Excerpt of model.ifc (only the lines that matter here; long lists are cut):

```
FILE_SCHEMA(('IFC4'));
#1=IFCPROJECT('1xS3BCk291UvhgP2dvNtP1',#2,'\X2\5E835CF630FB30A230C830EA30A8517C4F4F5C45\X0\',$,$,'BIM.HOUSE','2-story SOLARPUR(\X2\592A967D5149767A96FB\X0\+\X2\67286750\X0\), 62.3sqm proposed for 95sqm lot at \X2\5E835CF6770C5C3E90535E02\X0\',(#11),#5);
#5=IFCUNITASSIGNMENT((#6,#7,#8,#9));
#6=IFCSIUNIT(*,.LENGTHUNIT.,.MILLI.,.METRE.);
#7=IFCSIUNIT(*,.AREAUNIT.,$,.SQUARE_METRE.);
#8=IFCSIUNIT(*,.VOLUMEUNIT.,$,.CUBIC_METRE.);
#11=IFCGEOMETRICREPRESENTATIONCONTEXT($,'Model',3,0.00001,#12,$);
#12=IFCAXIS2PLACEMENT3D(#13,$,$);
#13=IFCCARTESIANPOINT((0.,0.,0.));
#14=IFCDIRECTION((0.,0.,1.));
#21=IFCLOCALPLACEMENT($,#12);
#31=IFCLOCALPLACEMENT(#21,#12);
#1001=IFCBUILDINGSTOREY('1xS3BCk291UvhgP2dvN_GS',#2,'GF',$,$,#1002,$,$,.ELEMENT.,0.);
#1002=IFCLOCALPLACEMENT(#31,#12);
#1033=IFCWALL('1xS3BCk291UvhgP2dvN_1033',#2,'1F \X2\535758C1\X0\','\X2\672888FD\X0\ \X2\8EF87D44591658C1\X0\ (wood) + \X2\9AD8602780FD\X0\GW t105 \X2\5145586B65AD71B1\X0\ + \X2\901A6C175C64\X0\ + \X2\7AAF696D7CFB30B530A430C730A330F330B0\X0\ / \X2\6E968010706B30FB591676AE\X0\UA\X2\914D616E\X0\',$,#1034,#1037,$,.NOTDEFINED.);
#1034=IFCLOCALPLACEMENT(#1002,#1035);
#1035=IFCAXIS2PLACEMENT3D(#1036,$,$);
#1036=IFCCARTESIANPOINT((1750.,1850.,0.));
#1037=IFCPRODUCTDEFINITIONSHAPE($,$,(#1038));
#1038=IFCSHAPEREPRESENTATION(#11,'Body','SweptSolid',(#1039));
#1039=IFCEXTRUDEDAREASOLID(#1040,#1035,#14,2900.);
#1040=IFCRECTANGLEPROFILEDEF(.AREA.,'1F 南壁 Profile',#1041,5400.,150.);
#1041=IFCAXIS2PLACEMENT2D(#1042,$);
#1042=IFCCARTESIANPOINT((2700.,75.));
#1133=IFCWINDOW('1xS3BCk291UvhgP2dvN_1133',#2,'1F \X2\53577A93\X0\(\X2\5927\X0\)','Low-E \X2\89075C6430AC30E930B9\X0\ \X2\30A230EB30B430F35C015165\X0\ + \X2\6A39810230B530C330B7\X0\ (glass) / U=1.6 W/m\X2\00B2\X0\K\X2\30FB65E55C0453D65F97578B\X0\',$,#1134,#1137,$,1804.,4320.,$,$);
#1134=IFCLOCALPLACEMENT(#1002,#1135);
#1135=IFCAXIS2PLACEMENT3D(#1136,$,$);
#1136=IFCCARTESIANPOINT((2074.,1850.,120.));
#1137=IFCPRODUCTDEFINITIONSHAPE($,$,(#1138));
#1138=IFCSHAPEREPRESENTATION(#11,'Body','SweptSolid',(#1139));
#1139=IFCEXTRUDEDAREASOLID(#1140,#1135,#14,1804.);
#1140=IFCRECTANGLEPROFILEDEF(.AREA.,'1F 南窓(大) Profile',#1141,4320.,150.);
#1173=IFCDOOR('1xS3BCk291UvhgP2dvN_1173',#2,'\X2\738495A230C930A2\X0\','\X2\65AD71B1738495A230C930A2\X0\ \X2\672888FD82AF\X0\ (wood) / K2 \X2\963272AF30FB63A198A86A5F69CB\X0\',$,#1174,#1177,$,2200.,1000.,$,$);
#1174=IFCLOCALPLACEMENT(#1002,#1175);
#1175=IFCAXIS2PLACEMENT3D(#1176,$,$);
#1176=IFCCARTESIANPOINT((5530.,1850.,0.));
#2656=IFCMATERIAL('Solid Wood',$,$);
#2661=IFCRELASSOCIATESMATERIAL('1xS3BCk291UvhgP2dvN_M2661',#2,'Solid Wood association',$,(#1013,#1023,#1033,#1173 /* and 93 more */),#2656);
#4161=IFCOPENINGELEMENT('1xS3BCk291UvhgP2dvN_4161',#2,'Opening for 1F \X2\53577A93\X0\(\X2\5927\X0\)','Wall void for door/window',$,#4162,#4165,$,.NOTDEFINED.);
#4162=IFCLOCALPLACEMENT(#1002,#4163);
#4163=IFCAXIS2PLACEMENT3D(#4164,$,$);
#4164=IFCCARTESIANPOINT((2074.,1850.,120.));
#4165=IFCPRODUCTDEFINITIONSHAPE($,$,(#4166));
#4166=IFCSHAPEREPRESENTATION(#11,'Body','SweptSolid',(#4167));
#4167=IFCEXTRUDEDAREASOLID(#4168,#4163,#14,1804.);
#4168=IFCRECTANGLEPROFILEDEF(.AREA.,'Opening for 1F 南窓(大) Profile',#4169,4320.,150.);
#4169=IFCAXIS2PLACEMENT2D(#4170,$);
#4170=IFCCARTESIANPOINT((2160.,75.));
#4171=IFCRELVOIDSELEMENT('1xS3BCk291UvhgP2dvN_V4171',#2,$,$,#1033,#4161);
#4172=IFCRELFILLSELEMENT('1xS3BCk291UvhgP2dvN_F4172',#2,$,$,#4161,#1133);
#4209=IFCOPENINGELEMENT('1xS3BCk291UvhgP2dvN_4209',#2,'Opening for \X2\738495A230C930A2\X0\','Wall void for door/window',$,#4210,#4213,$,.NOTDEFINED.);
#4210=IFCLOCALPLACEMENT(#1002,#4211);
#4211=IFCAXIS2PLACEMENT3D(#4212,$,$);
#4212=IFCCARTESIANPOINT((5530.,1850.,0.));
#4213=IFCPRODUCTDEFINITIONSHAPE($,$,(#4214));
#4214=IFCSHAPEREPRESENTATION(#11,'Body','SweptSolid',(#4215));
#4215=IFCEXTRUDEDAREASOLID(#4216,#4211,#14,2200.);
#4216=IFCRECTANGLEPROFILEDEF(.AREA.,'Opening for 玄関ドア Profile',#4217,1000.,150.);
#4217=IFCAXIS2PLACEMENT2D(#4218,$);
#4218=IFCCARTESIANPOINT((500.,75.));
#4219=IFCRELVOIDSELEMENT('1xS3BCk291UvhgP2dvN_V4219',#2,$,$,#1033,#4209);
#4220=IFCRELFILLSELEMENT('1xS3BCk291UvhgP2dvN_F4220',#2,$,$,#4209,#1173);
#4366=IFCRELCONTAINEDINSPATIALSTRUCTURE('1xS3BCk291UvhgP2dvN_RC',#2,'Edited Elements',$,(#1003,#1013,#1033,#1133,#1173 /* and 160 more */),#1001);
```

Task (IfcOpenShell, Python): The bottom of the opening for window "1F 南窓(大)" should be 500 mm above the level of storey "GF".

```python
import numpy as np
import ifcopenshell
import ifcopenshell.api.geometry
import ifcopenshell.geom
import ifcopenshell.util.element
import ifcopenshell.util.placement
import ifcopenshell.util.shape
import ifcopenshell.util.unit

model = ifcopenshell.open("model.ifc")
unit_scale = ifcopenshell.util.unit.calculate_unit_scale(model)

window = model.by_id(1133)
opening = window.FillsVoids[0].RelatingOpeningElement
storey = ifcopenshell.util.element.get_container(window, ifc_class="IfcBuildingStorey")
level = ifcopenshell.util.placement.get_local_placement(storey.ObjectPlacement)[2, 3]

# The opening's origin need not be at the sill, so measure its lowest point.
shape = ifcopenshell.geom.create_shape(ifcopenshell.geom.settings(), opening)
bottom = ifcopenshell.util.shape.get_shape_bottom_elevation(shape, shape.geometry) / unit_scale
dz = level + 0.5 / unit_scale - bottom

shift = np.array([0.0, 0.0, dz])
# The window is not placed relative to its opening, so move both.
for product in (opening, window):
    matrix = ifcopenshell.util.placement.get_local_placement(product.ObjectPlacement)
    matrix[:3, 3] += shift
    ifcopenshell.api.geometry.edit_object_placement(model, product=product, matrix=matrix, is_si=False)

print(f"moved by {dz * unit_scale:+.3f} m")

model.write("model-out.ifc")
```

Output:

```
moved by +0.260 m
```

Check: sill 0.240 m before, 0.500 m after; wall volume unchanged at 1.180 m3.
